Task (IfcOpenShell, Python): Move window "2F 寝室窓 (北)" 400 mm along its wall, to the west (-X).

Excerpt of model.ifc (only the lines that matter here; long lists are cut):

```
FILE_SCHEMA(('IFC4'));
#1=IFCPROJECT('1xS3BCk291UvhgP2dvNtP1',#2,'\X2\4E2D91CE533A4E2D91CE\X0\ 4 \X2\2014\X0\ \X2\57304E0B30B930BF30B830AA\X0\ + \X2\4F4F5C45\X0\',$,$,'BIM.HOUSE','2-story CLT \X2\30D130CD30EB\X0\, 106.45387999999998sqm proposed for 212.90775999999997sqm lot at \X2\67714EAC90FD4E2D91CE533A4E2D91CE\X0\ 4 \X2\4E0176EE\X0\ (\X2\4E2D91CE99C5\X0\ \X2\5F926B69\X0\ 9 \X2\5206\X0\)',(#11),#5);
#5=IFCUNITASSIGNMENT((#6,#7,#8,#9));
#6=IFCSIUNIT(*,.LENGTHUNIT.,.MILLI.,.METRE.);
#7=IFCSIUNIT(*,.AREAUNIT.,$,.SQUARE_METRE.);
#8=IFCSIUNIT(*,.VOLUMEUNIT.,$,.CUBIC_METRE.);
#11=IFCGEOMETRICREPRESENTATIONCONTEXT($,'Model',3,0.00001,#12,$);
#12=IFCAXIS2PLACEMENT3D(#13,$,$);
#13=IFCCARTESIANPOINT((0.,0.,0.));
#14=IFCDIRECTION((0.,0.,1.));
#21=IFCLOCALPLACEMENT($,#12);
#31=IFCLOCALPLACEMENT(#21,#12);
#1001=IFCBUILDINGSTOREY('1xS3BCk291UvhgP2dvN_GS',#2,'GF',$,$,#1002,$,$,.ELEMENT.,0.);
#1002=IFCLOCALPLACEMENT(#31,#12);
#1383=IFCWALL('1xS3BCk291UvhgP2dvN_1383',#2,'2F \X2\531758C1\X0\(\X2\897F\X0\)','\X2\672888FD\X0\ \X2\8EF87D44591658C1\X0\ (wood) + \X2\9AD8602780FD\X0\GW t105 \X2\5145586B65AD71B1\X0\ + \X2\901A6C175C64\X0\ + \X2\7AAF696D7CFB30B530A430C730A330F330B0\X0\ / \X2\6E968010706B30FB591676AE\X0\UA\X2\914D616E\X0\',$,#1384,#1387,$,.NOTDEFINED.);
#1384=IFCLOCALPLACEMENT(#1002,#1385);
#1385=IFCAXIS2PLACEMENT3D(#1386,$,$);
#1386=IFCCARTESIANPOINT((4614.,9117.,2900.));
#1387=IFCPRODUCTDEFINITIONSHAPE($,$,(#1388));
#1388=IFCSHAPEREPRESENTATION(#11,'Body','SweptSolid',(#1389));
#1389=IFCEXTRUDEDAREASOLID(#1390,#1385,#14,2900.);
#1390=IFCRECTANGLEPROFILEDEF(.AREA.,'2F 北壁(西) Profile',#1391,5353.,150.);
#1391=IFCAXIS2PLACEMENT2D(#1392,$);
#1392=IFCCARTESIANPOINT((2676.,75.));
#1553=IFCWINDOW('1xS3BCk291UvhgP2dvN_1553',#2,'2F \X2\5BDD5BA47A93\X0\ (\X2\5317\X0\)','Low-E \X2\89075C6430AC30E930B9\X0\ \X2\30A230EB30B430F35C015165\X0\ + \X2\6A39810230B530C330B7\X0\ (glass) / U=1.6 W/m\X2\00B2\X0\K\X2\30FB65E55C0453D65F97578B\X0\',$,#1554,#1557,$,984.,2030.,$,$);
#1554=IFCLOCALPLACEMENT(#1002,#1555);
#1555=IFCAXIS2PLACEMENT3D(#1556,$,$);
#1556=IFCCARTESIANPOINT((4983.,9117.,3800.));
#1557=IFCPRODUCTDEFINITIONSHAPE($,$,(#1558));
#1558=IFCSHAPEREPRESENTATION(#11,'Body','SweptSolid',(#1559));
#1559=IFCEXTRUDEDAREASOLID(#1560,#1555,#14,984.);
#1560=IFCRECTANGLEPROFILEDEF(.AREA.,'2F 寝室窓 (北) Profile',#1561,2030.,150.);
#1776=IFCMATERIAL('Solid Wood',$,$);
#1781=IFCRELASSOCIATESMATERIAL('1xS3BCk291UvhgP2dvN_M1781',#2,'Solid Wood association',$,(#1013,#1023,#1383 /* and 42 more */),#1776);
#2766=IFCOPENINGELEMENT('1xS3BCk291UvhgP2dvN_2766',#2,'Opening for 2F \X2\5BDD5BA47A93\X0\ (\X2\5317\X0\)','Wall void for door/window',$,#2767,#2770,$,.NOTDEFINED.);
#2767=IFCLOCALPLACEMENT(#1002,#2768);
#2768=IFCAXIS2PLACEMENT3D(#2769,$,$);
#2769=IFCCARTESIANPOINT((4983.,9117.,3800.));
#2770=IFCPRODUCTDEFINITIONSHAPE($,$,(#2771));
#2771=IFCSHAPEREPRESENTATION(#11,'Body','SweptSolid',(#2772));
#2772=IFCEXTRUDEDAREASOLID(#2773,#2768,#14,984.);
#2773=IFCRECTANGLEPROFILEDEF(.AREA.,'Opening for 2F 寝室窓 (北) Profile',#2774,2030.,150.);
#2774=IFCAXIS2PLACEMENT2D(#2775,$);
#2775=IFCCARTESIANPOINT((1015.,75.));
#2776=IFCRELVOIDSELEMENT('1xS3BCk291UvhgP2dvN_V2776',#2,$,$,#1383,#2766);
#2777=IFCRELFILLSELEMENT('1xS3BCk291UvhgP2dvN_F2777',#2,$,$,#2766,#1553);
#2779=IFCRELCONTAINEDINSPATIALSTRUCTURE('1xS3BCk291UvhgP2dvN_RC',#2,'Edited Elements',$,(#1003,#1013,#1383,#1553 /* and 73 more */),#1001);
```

```python
import ifcopenshell
import ifcopenshell.api.geometry
import ifcopenshell.util.placement
import ifcopenshell.util.unit

model = ifcopenshell.open("model.ifc")
unit_scale = ifcopenshell.util.unit.calculate_unit_scale(model)

window = model.by_guid("1xS3BCk291UvhgP2dvN_1553")
opening = window.FillsVoids[0].RelatingOpeningElement
wall = opening.VoidsElements[0].RelatingBuildingElement

wall_matrix = ifcopenshell.util.placement.get_local_placement(wall.ObjectPlacement)
shift = wall_matrix[:3, 0] * -0.4 / unit_scale
before = ifcopenshell.util.placement.get_local_placement(window.ObjectPlacement)[:3, 3].copy()

# The window is not placed relative to its opening, so move both.
for product in (opening, window):
    matrix = ifcopenshell.util.placement.get_local_placement(product.ObjectPlacement)
    matrix[:3, 3] += shift
    ifcopenshell.api.geometry.edit_object_placement(model, product=product, matrix=matrix, is_si=False)

after = ifcopenshell.util.placement.get_local_placement(window.ObjectPlacement)[:3, 3]
print("window moved by", (after - before).round(3) + 0.0)

model.write("model-out.ifc")
```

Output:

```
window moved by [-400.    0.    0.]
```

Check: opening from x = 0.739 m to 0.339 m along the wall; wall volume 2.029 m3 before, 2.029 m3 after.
